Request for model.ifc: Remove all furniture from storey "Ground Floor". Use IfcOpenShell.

First a look at what the model holds.

```python
import ifcopenshell
import ifcopenshell.util.element

model = ifcopenshell.open("model.ifc")
print(model.schema)
storey = next(s for s in model.by_type("IfcBuildingStorey") if s.Name == "Ground Floor")
furniture = [e for e in ifcopenshell.util.element.get_decomposition(storey) if e.is_a("IfcFurnishingElement")]
seen = {}
for e in furniture:
    element_type = ifcopenshell.util.element.get_type(e)
    name = element_type.Name if element_type not in (None, e) else None
    seen[name] = seen.get(name, 0) + 1
for name, count in sorted(seen.items(), key=str):
    print(count, "x", name)
```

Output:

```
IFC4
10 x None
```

```python
import ifcopenshell
import ifcopenshell.api.root
import ifcopenshell.util.element

model = ifcopenshell.open("model.ifc")

storey = next(s for s in model.by_type("IfcBuildingStorey") if s.Name == "Ground Floor")
furniture = [e for e in ifcopenshell.util.element.get_decomposition(storey) if e.is_a("IfcFurnishingElement")]

for e in furniture:
    ifcopenshell.api.root.remove_product(model, product=e)
print(len(furniture), "removed")

model.write("model_updated.ifc")
```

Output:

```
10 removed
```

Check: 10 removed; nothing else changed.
